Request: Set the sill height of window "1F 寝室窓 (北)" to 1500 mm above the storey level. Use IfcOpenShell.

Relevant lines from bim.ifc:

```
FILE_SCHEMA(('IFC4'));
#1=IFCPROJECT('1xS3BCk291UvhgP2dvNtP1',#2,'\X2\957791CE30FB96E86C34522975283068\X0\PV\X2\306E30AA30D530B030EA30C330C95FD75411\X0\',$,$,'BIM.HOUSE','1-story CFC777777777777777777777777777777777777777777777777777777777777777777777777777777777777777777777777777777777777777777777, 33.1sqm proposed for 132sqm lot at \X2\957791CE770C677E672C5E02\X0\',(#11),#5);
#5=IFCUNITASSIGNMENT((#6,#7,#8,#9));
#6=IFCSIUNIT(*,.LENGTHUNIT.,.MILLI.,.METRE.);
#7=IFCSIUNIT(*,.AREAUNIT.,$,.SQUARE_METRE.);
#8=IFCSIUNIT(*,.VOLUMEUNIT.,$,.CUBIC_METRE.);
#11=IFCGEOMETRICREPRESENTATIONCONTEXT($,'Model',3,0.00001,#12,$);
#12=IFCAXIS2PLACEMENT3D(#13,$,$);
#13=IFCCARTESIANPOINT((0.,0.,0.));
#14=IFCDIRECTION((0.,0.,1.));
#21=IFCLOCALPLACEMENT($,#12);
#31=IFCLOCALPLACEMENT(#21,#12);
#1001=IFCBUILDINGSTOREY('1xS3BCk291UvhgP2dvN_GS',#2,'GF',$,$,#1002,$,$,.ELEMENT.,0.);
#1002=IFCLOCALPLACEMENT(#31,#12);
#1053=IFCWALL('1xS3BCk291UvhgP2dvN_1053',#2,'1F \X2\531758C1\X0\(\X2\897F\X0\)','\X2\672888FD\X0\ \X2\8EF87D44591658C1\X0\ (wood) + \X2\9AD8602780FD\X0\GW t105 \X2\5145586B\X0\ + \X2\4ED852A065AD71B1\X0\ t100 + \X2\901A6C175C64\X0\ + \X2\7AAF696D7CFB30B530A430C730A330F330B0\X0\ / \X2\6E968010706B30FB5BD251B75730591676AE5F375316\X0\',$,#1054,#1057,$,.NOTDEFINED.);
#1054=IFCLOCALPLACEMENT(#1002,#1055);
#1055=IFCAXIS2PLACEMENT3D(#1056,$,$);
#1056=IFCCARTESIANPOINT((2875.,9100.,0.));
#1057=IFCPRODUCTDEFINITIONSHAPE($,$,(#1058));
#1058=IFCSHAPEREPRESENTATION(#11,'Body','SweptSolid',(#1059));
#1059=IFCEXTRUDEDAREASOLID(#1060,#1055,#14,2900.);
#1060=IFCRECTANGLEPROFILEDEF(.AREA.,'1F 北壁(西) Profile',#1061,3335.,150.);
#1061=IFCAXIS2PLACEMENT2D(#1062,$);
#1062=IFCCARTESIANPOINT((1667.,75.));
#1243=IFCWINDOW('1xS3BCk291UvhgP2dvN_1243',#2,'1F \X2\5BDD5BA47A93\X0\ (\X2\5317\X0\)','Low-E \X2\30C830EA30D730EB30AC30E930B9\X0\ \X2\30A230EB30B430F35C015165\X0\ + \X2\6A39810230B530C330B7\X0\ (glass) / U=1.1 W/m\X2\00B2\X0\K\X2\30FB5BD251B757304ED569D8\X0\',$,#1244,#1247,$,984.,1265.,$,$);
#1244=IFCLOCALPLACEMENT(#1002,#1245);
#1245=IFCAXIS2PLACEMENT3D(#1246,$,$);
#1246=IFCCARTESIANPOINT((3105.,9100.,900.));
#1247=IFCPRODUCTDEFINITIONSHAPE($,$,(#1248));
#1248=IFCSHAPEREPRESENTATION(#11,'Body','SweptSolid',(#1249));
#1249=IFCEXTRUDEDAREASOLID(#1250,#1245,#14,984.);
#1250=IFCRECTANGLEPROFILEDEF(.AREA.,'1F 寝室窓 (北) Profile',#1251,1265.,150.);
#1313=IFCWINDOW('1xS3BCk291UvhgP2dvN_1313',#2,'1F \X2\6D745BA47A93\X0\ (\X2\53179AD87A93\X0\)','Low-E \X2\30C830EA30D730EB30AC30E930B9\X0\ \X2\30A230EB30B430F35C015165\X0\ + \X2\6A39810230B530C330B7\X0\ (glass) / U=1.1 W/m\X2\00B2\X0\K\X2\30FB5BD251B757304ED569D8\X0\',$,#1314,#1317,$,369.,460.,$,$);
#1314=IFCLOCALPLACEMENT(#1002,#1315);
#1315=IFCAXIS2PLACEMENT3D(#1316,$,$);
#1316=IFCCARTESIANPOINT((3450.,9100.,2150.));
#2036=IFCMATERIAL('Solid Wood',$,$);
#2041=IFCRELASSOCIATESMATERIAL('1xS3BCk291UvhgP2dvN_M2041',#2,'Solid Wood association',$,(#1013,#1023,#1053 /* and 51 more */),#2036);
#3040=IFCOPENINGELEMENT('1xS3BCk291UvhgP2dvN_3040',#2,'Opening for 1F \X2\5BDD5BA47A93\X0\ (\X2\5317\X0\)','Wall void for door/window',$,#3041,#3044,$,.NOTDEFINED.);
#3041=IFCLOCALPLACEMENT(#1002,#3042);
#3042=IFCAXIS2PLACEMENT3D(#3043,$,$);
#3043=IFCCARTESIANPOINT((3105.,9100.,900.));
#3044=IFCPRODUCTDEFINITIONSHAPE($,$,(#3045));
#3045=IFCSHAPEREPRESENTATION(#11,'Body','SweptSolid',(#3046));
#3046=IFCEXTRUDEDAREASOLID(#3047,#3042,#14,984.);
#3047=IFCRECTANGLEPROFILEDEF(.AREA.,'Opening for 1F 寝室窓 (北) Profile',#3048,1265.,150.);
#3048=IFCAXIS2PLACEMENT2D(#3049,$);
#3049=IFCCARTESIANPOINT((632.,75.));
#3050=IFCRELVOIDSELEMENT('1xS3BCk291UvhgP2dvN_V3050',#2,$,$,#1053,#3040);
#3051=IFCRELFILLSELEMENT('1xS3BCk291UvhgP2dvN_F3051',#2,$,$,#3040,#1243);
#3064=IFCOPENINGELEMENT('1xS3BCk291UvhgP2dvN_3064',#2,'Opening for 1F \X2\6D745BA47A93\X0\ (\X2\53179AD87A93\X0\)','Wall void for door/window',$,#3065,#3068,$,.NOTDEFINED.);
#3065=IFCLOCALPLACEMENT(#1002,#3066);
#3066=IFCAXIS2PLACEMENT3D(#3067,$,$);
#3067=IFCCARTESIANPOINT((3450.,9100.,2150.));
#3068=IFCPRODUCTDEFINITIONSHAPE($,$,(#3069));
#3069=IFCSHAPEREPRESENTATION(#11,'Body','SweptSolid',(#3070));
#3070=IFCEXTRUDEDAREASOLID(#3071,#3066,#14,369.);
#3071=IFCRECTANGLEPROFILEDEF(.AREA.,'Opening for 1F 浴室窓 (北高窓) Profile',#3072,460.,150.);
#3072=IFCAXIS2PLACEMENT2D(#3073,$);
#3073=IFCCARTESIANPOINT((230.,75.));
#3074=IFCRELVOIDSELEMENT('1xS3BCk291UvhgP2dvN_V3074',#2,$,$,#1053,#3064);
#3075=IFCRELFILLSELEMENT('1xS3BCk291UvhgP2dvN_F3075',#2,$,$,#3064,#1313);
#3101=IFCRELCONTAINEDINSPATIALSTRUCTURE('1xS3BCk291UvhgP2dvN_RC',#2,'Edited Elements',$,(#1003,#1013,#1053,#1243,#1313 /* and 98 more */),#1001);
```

```python
import numpy as np
import ifcopenshell
import ifcopenshell.api.geometry
import ifcopenshell.geom
import ifcopenshell.util.element
import ifcopenshell.util.placement
import ifcopenshell.util.shape
import ifcopenshell.util.unit

model = ifcopenshell.open("bim.ifc")
unit_scale = ifcopenshell.util.unit.calculate_unit_scale(model)

window = model.by_guid("1xS3BCk291UvhgP2dvN_1243")
opening = window.FillsVoids[0].RelatingOpeningElement
storey = ifcopenshell.util.element.get_container(window, ifc_class="IfcBuildingStorey")
level = ifcopenshell.util.placement.get_local_placement(storey.ObjectPlacement)[2, 3]

# The opening's origin need not be at the sill, so measure its lowest point.
shape = ifcopenshell.geom.create_shape(ifcopenshell.geom.settings(), opening)
bottom = ifcopenshell.util.shape.get_shape_bottom_elevation(shape, shape.geometry) / unit_scale
dz = level + 1.5 / unit_scale - bottom

shift = np.array([0.0, 0.0, dz])
# The window is not placed relative to its opening, so move both.
for product in (opening, window):
    matrix = ifcopenshell.util.placement.get_local_placement(product.ObjectPlacement)
    matrix[:3, 3] += shift
    ifcopenshell.api.geometry.edit_object_placement(model, product=product, matrix=matrix, is_si=False)

print(f"moved by {dz * unit_scale:+.3f} m")

model.write("bim_edited.ifc")
```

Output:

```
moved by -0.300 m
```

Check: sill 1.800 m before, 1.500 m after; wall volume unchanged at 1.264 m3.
